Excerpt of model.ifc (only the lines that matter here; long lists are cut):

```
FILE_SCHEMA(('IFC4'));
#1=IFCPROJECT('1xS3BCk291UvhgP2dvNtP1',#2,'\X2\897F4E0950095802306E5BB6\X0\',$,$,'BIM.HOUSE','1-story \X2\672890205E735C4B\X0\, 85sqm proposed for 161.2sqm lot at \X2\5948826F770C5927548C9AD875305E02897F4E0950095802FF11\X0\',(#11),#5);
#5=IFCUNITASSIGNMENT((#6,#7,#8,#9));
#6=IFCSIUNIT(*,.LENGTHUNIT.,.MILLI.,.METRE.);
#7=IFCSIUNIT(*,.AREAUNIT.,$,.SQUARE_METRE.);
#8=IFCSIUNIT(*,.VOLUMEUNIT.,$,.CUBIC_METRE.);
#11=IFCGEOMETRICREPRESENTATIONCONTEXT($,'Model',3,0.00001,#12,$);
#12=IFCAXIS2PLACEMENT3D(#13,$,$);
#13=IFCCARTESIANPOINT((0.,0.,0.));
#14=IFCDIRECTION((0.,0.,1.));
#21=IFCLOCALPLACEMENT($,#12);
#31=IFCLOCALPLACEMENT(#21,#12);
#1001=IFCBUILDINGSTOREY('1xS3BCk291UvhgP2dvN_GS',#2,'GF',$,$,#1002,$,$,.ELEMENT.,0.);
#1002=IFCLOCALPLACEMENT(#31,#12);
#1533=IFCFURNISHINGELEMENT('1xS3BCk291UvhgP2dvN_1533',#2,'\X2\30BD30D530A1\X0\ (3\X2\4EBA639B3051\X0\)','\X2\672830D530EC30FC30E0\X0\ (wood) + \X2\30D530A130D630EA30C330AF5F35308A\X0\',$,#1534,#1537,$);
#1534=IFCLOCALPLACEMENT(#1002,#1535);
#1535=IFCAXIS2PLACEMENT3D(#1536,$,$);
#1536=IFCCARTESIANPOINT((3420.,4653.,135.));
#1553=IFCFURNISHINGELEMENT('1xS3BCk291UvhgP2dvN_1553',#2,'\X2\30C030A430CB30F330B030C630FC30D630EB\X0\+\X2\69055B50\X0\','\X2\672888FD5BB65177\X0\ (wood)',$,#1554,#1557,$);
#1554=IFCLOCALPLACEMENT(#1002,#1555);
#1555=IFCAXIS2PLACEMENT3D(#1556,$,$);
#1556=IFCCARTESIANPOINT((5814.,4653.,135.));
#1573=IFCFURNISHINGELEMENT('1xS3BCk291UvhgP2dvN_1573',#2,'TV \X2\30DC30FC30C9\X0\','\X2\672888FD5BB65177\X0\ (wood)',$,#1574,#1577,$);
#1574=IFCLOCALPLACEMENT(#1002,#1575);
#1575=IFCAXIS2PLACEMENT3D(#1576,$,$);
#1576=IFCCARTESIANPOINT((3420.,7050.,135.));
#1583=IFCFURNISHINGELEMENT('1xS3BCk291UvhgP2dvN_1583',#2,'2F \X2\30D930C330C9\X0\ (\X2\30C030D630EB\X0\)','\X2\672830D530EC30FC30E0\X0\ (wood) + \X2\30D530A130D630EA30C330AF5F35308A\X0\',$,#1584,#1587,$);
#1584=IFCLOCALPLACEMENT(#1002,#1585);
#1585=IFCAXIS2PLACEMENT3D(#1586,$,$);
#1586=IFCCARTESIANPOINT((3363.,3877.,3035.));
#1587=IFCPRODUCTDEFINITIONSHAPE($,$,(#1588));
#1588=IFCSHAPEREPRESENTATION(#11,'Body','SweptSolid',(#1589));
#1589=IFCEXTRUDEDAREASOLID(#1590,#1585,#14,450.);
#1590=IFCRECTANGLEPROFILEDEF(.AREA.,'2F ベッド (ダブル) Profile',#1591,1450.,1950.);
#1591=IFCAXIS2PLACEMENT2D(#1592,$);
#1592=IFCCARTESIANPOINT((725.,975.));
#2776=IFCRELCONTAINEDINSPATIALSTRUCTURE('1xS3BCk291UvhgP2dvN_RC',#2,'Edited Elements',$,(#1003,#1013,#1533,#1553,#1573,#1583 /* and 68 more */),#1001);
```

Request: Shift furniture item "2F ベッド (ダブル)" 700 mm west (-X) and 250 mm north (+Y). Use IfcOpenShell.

```python
import ifcopenshell
import ifcopenshell.api.geometry
import ifcopenshell.util.placement
import ifcopenshell.util.unit

model = ifcopenshell.open("model.ifc")
unit_scale = ifcopenshell.util.unit.calculate_unit_scale(model)

item = model.by_guid("1xS3BCk291UvhgP2dvN_1583")
matrix = ifcopenshell.util.placement.get_local_placement(item.ObjectPlacement)
matrix[0, 3] -= 0.7 / unit_scale
matrix[1, 3] += 0.25 / unit_scale
ifcopenshell.api.geometry.edit_object_placement(model, product=item, matrix=matrix, is_si=False)

print(ifcopenshell.util.placement.get_local_placement(item.ObjectPlacement).round(3) + 0.0)

model.write("model_updated.ifc")
```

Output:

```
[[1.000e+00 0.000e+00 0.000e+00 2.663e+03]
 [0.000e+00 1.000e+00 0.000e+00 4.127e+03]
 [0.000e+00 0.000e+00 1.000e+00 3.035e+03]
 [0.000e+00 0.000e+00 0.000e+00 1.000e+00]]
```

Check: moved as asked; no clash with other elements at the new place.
